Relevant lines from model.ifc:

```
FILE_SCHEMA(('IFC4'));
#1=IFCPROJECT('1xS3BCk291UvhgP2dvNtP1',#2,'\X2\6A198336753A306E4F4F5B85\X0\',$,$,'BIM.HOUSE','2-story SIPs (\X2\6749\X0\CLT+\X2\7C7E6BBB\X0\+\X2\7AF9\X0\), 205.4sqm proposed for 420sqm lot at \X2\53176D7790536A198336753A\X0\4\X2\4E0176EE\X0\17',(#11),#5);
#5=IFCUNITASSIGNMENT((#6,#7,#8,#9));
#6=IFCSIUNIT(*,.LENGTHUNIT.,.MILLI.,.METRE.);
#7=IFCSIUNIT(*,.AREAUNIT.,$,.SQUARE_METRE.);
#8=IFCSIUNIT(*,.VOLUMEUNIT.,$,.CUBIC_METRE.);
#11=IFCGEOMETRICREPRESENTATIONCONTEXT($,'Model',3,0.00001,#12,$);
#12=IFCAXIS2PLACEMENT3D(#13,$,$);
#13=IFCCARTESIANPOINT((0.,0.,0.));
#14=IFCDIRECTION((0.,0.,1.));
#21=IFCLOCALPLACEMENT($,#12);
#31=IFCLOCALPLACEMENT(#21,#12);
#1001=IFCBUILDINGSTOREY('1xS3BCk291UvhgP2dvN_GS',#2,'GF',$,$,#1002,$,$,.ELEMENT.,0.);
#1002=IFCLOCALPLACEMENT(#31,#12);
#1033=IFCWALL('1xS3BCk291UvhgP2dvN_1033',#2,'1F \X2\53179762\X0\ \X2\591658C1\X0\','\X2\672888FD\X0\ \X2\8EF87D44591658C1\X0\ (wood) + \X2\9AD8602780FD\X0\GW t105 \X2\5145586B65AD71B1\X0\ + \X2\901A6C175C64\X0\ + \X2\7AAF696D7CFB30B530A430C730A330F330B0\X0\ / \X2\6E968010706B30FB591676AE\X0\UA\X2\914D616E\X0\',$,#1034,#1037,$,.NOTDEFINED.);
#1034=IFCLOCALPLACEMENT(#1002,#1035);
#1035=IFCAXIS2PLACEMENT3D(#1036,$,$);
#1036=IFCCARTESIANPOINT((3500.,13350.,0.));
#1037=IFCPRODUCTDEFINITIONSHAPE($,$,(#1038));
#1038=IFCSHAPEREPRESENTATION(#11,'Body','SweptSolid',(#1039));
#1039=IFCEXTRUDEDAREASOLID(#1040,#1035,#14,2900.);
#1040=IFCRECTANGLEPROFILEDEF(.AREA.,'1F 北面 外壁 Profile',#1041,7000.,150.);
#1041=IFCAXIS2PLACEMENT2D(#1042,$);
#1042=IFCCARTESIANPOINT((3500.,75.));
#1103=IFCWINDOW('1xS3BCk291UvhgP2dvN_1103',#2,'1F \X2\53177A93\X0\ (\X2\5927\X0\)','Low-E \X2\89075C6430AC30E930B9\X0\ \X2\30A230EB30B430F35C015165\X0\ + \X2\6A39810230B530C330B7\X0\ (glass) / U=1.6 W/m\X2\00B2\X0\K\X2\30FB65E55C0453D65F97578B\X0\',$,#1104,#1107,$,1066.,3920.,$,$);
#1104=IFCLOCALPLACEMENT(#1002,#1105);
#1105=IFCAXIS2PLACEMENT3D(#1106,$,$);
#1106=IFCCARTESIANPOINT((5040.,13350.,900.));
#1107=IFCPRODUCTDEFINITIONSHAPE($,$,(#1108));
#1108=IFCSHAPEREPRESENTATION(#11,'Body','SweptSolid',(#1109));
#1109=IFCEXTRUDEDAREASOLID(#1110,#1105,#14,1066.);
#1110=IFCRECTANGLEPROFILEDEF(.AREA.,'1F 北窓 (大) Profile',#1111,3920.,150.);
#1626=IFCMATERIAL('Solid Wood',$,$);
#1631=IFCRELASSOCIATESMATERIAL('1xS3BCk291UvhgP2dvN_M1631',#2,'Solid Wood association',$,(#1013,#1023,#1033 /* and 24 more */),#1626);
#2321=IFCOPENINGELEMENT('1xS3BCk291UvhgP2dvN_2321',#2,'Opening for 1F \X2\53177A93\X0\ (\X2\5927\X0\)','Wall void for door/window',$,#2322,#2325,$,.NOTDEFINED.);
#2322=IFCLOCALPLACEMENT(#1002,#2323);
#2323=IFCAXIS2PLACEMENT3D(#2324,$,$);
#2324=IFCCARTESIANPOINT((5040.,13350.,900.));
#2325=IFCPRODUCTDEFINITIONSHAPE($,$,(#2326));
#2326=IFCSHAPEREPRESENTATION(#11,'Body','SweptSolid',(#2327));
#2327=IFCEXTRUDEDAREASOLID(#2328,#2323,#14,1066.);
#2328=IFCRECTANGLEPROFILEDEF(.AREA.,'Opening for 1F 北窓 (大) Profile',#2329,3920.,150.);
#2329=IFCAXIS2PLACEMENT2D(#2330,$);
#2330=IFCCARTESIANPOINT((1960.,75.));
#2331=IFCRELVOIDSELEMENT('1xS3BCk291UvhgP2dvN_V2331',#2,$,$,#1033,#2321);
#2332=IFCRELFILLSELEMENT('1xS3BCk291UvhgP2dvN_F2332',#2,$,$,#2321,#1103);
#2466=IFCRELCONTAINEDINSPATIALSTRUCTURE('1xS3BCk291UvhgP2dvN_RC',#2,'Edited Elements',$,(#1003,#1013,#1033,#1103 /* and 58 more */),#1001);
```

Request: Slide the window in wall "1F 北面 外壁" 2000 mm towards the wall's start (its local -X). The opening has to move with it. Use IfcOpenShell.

```python
import ifcopenshell
import ifcopenshell.api.geometry
import ifcopenshell.util.placement

model = ifcopenshell.open("model.ifc")

window = model.by_guid("1xS3BCk291UvhgP2dvN_1103")
opening = window.FillsVoids[0].RelatingOpeningElement
wall = opening.VoidsElements[0].RelatingBuildingElement

wall_matrix = ifcopenshell.util.placement.get_local_placement(wall.ObjectPlacement)
shift = wall_matrix[:3, 0] * -2000.0
before = ifcopenshell.util.placement.get_local_placement(window.ObjectPlacement)[:3, 3].copy()

# The window is not placed relative to its opening, so move both.
for product in (opening, window):
    matrix = ifcopenshell.util.placement.get_local_placement(product.ObjectPlacement)
    matrix[:3, 3] += shift
    ifcopenshell.api.geometry.edit_object_placement(model, product=product, matrix=matrix, is_si=False)

after = ifcopenshell.util.placement.get_local_placement(window.ObjectPlacement)[:3, 3]
print("window moved by", (after - before).round(3) + 0.0)

model.write("model_edited.ifc")
```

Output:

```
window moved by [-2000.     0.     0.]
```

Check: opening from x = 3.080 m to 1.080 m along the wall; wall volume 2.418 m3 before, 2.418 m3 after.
